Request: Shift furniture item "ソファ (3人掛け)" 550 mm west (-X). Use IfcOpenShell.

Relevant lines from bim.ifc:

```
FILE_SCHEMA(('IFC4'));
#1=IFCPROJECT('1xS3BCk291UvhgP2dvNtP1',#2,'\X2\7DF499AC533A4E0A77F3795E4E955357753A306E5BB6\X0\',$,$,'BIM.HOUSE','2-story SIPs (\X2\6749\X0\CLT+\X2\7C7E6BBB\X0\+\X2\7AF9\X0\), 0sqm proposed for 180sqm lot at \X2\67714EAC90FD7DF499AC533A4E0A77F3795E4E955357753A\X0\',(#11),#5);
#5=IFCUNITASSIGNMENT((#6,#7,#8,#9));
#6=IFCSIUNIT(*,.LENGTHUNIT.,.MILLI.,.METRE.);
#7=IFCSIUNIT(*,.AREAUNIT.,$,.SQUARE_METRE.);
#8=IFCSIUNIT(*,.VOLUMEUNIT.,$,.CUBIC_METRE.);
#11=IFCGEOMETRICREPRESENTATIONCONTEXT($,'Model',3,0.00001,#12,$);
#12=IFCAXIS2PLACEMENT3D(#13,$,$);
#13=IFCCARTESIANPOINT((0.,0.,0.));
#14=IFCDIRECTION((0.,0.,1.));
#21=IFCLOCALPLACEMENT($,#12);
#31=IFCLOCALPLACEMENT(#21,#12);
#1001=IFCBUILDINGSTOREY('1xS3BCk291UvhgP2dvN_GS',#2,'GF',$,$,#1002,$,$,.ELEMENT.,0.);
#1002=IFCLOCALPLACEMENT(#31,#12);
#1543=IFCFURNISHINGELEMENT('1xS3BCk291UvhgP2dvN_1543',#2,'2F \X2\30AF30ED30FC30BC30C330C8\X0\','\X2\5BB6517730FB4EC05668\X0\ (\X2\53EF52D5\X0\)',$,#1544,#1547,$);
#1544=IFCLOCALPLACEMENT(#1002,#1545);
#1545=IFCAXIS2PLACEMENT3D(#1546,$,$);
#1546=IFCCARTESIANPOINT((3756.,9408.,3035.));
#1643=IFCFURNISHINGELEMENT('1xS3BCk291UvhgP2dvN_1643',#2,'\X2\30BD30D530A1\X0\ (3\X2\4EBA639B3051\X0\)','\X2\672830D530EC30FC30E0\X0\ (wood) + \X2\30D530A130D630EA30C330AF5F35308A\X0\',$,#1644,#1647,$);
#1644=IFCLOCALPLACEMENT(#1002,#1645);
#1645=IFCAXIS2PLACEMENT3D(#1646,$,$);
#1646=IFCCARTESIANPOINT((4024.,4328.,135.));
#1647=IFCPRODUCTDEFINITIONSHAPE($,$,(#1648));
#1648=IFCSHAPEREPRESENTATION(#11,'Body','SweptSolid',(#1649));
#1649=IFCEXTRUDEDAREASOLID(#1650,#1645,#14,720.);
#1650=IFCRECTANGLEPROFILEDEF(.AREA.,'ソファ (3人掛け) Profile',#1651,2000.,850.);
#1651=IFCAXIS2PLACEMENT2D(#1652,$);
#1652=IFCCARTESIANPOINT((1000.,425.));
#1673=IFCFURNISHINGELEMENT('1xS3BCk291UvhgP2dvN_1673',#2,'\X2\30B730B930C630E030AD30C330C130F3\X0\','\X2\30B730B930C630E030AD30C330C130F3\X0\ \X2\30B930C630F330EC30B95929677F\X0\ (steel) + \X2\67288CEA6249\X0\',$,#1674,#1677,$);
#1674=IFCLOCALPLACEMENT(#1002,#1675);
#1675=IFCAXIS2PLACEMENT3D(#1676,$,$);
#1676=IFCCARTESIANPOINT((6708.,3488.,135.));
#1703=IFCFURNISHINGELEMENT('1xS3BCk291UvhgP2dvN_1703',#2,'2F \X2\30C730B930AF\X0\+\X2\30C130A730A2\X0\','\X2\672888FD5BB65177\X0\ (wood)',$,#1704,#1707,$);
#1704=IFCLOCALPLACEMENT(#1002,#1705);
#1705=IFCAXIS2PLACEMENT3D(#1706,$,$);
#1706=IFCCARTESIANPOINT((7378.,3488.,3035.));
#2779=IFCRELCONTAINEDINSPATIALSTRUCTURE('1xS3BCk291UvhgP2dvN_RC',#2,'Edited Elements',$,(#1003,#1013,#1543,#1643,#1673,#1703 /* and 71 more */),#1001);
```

```python
import ifcopenshell
import ifcopenshell.api.geometry
import ifcopenshell.util.placement
import ifcopenshell.util.unit

model = ifcopenshell.open("bim.ifc")
unit_scale = ifcopenshell.util.unit.calculate_unit_scale(model)

item = model.by_guid("1xS3BCk291UvhgP2dvN_1643")
matrix = ifcopenshell.util.placement.get_local_placement(item.ObjectPlacement)
matrix[0, 3] -= 0.55 / unit_scale
ifcopenshell.api.geometry.edit_object_placement(model, product=item, matrix=matrix, is_si=False)

print(ifcopenshell.util.placement.get_local_placement(item.ObjectPlacement).round(3) + 0.0)

model.write("bim_edited.ifc")
```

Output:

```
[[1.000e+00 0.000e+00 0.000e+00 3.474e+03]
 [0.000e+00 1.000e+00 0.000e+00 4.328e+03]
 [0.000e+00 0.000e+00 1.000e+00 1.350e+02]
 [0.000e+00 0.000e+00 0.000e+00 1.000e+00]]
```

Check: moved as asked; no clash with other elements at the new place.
